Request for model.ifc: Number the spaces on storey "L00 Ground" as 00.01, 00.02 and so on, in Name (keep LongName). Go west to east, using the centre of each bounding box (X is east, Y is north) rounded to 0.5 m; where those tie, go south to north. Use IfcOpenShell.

First a look at what the model holds.

```python
import ifcopenshell
import ifcopenshell.util.element
import ifcopenshell.util.placement

model = ifcopenshell.open("model.ifc")
print(model.schema)
storey = next(s for s in model.by_type("IfcBuildingStorey") if s.Name == "L00 Ground")
spaces = [e for e in ifcopenshell.util.element.get_decomposition(storey) if e.is_a("IfcSpace")]
for e in sorted(spaces, key=lambda e: e.id()):
    origin = ifcopenshell.util.placement.get_local_placement(e.ObjectPlacement)[:3, 3]
    print(e.id(), e.Name, e.LongName, origin.round(2) + 0.0, sep=" | ")
```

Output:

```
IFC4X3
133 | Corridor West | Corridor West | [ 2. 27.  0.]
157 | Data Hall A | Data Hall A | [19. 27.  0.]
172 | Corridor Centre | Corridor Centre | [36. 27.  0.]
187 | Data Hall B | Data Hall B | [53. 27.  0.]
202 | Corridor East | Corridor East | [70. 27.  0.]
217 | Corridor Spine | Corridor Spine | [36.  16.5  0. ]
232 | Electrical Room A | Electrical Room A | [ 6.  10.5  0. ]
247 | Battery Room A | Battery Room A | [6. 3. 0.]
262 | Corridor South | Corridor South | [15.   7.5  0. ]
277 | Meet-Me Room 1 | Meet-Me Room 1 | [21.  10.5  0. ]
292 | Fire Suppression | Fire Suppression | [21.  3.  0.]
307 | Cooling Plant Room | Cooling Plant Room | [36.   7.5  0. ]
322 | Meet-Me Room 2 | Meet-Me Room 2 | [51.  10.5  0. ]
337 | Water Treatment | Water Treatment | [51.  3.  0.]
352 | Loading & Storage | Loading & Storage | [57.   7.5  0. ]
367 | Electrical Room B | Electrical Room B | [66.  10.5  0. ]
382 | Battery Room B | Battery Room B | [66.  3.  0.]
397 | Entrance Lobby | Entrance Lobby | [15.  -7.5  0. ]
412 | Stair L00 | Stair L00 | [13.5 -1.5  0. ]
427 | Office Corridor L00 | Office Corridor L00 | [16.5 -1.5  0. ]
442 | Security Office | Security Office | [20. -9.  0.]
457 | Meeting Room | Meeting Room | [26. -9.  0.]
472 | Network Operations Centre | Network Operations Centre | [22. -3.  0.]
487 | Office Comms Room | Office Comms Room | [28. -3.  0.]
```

```python
import ifcopenshell
import ifcopenshell.geom
import ifcopenshell.util.element
import ifcopenshell.util.shape

model = ifcopenshell.open("model.ifc")
settings = ifcopenshell.geom.settings()
settings.set("use-world-coords", True)


def centre(element):
    shape = ifcopenshell.geom.create_shape(settings, element)
    return ifcopenshell.util.shape.get_bbox_centroid(shape.geometry)


storey = next(s for s in model.by_type("IfcBuildingStorey") if s.Name == "L00 Ground")
spaces = [e for e in ifcopenshell.util.element.get_decomposition(storey) if e.is_a("IfcSpace")]

# Insertion points can sit at a corner or the storey origin, so sort by the geometry (in metres).
centres = {e: centre(e) for e in spaces}
spaces.sort(key=lambda e: (round(centres[e][0] / 0.5), centres[e][1]))

for i, e in enumerate(spaces, start=1):
    number = f"00.{i:02d}"
    e.Name = number
    print(e.id(), number)

model.write("model_v2.ifc")
```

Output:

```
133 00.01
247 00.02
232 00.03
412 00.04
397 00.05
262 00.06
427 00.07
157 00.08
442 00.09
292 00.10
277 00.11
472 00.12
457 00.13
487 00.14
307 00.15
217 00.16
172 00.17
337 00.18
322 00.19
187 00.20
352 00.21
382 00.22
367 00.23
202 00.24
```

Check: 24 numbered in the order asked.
